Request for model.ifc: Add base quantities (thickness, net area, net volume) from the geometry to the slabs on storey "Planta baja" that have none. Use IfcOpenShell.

First a look at what the model holds.

```python
import ifcopenshell
import ifcopenshell.util.element
import ifcopenshell.util.unit

model = ifcopenshell.open("model.ifc")
print(model.schema)
for unit_type in ("LENGTHUNIT", "AREAUNIT", "VOLUMEUNIT"):
    print(unit_type, ifcopenshell.util.unit.calculate_unit_scale(model, unit_type))
storey = next(s for s in model.by_type("IfcBuildingStorey") if s.Name == "Planta baja")
slabs = [e for e in ifcopenshell.util.element.get_decomposition(storey) if e.is_a("IfcSlab")]
for e in sorted(slabs, key=lambda e: e.id()):
    print(e.id(), e.is_a(), e.Name, list(ifcopenshell.util.element.get_psets(e, qtos_only=True)), sep=" | ")
```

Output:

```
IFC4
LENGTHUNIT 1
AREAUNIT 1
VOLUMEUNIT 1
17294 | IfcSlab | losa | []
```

```python
import ifcopenshell
import ifcopenshell.api.pset
import ifcopenshell.geom
import ifcopenshell.util.element
import ifcopenshell.util.shape
import ifcopenshell.util.unit

model = ifcopenshell.open("model.ifc")
unit_scale = ifcopenshell.util.unit.calculate_unit_scale(model)
area_scale = ifcopenshell.util.unit.calculate_unit_scale(model, "AREAUNIT")
volume_scale = ifcopenshell.util.unit.calculate_unit_scale(model, "VOLUMEUNIT")
settings = ifcopenshell.geom.settings()

storey = next(s for s in model.by_type("IfcBuildingStorey") if s.Name == "Planta baja")
slabs = [e for e in ifcopenshell.util.element.get_decomposition(storey) if e.is_a("IfcSlab")]

for e in sorted(slabs, key=lambda e: e.id()):
    if ifcopenshell.util.element.get_psets(e, qtos_only=True, should_inherit=False):
        continue
    # Geometry comes back in metres, in the element's own axes.
    shape = ifcopenshell.geom.create_shape(settings, e)
    values = {
        "Width": ifcopenshell.util.shape.get_z(shape.geometry) / unit_scale,
        "NetArea": ifcopenshell.util.shape.get_footprint_area(shape.geometry) / area_scale,
        "NetVolume": ifcopenshell.util.shape.get_volume(shape.geometry) / volume_scale,
    }
    qto = ifcopenshell.api.pset.add_qto(model, product=e, name="Qto_SlabBaseQuantities")
    ifcopenshell.api.pset.edit_qto(model, qto=qto, properties=values)
    print(e.id(), {k: round(v, 3) for k, v in values.items()})

model.write("model_rev.ifc")
```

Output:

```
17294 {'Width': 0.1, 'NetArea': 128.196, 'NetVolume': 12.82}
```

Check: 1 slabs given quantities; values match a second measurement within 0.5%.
